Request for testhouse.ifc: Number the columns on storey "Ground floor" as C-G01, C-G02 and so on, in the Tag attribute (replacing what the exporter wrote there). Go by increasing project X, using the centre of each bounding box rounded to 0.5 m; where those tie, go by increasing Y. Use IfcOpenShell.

First a look at what the model holds.

```python
import ifcopenshell
import ifcopenshell.util.element
import ifcopenshell.util.placement

model = ifcopenshell.open("testhouse.ifc")
print(model.schema)
storey = next(s for s in model.by_type("IfcBuildingStorey") if s.Name == "Ground floor")
columns = [e for e in ifcopenshell.util.element.get_decomposition(storey) if e.is_a("IfcColumn")]
for e in sorted(columns, key=lambda e: e.id()):
    origin = ifcopenshell.util.placement.get_local_placement(e.ObjectPlacement)[:3, 3]
    print(e.id(), e.Tag, e.Name, origin.round(2) + 0.0, sep=" | ")
```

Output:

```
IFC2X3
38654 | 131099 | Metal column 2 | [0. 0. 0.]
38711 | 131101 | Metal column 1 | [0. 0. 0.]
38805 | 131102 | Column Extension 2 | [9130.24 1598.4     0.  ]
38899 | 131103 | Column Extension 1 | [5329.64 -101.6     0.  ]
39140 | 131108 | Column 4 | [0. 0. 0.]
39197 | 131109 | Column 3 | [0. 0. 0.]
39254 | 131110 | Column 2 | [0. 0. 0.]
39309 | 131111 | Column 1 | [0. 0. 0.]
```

```python
import ifcopenshell
import ifcopenshell.geom
import ifcopenshell.util.element
import ifcopenshell.util.shape

model = ifcopenshell.open("testhouse.ifc")
settings = ifcopenshell.geom.settings()
settings.set("use-world-coords", True)


def centre(element):
    shape = ifcopenshell.geom.create_shape(settings, element)
    return ifcopenshell.util.shape.get_bbox_centroid(shape.geometry)


storey = next(s for s in model.by_type("IfcBuildingStorey") if s.Name == "Ground floor")
columns = [e for e in ifcopenshell.util.element.get_decomposition(storey) if e.is_a("IfcColumn")]

# Insertion points can sit at a corner or the storey origin, so sort by the geometry (in metres).
centres = {e: centre(e) for e in columns}
columns.sort(key=lambda e: (round(centres[e][0] / 0.5), centres[e][1]))

for i, e in enumerate(columns, start=1):
    number = f"C-G{i:02d}"
    e.Tag = number
    print(e.id(), number)

model.write("testhouse_rev.ifc")
```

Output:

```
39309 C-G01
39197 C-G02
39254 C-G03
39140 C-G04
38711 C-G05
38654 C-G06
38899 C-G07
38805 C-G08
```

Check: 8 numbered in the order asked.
